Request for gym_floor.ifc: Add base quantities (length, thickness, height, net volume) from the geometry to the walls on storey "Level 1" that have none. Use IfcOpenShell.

First a look at what the model holds.

```python
import ifcopenshell
import ifcopenshell.util.element
import ifcopenshell.util.unit

model = ifcopenshell.open("gym_floor.ifc")
print(model.schema)
for unit_type in ("LENGTHUNIT", "AREAUNIT", "VOLUMEUNIT"):
    print(unit_type, ifcopenshell.util.unit.calculate_unit_scale(model, unit_type))
storey = next(s for s in model.by_type("IfcBuildingStorey") if s.Name == "Level 1")
walls = [e for e in ifcopenshell.util.element.get_decomposition(storey) if e.is_a("IfcWall")]
for e in sorted(walls, key=lambda e: e.id()):
    print(e.id(), e.is_a(), e.Name, list(ifcopenshell.util.element.get_psets(e, qtos_only=True)), sep=" | ")
```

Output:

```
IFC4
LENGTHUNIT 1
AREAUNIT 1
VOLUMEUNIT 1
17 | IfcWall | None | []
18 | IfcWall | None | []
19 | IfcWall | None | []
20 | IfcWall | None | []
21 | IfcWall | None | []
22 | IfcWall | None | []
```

```python
import ifcopenshell
import ifcopenshell.api.pset
import ifcopenshell.geom
import ifcopenshell.util.element
import ifcopenshell.util.shape
import ifcopenshell.util.unit

model = ifcopenshell.open("gym_floor.ifc")
unit_scale = ifcopenshell.util.unit.calculate_unit_scale(model)
volume_scale = ifcopenshell.util.unit.calculate_unit_scale(model, "VOLUMEUNIT")
settings = ifcopenshell.geom.settings()

storey = next(s for s in model.by_type("IfcBuildingStorey") if s.Name == "Level 1")
walls = [e for e in ifcopenshell.util.element.get_decomposition(storey) if e.is_a("IfcWall")]

for e in sorted(walls, key=lambda e: e.id()):
    if ifcopenshell.util.element.get_psets(e, qtos_only=True, should_inherit=False):
        continue
    # Geometry comes back in metres, in the element's own axes.
    shape = ifcopenshell.geom.create_shape(settings, e)
    values = {
        "Length": ifcopenshell.util.shape.get_x(shape.geometry) / unit_scale,
        "Width": ifcopenshell.util.shape.get_y(shape.geometry) / unit_scale,
        "Height": ifcopenshell.util.shape.get_z(shape.geometry) / unit_scale,
        "NetVolume": ifcopenshell.util.shape.get_volume(shape.geometry) / volume_scale,
    }
    qto = ifcopenshell.api.pset.add_qto(model, product=e, name="Qto_WallBaseQuantities")
    ifcopenshell.api.pset.edit_qto(model, qto=qto, properties=values)
    print(e.id(), {k: round(v, 3) for k, v in values.items()})

model.write("gym_floor_updated.ifc")
```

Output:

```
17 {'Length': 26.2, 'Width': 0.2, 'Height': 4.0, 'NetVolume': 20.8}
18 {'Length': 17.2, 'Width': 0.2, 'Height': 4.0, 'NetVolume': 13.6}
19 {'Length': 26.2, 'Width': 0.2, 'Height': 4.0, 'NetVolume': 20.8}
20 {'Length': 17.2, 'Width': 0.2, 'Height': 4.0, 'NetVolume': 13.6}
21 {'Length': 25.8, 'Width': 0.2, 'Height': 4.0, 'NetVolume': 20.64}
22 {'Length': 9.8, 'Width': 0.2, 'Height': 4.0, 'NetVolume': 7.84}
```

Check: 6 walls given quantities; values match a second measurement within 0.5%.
